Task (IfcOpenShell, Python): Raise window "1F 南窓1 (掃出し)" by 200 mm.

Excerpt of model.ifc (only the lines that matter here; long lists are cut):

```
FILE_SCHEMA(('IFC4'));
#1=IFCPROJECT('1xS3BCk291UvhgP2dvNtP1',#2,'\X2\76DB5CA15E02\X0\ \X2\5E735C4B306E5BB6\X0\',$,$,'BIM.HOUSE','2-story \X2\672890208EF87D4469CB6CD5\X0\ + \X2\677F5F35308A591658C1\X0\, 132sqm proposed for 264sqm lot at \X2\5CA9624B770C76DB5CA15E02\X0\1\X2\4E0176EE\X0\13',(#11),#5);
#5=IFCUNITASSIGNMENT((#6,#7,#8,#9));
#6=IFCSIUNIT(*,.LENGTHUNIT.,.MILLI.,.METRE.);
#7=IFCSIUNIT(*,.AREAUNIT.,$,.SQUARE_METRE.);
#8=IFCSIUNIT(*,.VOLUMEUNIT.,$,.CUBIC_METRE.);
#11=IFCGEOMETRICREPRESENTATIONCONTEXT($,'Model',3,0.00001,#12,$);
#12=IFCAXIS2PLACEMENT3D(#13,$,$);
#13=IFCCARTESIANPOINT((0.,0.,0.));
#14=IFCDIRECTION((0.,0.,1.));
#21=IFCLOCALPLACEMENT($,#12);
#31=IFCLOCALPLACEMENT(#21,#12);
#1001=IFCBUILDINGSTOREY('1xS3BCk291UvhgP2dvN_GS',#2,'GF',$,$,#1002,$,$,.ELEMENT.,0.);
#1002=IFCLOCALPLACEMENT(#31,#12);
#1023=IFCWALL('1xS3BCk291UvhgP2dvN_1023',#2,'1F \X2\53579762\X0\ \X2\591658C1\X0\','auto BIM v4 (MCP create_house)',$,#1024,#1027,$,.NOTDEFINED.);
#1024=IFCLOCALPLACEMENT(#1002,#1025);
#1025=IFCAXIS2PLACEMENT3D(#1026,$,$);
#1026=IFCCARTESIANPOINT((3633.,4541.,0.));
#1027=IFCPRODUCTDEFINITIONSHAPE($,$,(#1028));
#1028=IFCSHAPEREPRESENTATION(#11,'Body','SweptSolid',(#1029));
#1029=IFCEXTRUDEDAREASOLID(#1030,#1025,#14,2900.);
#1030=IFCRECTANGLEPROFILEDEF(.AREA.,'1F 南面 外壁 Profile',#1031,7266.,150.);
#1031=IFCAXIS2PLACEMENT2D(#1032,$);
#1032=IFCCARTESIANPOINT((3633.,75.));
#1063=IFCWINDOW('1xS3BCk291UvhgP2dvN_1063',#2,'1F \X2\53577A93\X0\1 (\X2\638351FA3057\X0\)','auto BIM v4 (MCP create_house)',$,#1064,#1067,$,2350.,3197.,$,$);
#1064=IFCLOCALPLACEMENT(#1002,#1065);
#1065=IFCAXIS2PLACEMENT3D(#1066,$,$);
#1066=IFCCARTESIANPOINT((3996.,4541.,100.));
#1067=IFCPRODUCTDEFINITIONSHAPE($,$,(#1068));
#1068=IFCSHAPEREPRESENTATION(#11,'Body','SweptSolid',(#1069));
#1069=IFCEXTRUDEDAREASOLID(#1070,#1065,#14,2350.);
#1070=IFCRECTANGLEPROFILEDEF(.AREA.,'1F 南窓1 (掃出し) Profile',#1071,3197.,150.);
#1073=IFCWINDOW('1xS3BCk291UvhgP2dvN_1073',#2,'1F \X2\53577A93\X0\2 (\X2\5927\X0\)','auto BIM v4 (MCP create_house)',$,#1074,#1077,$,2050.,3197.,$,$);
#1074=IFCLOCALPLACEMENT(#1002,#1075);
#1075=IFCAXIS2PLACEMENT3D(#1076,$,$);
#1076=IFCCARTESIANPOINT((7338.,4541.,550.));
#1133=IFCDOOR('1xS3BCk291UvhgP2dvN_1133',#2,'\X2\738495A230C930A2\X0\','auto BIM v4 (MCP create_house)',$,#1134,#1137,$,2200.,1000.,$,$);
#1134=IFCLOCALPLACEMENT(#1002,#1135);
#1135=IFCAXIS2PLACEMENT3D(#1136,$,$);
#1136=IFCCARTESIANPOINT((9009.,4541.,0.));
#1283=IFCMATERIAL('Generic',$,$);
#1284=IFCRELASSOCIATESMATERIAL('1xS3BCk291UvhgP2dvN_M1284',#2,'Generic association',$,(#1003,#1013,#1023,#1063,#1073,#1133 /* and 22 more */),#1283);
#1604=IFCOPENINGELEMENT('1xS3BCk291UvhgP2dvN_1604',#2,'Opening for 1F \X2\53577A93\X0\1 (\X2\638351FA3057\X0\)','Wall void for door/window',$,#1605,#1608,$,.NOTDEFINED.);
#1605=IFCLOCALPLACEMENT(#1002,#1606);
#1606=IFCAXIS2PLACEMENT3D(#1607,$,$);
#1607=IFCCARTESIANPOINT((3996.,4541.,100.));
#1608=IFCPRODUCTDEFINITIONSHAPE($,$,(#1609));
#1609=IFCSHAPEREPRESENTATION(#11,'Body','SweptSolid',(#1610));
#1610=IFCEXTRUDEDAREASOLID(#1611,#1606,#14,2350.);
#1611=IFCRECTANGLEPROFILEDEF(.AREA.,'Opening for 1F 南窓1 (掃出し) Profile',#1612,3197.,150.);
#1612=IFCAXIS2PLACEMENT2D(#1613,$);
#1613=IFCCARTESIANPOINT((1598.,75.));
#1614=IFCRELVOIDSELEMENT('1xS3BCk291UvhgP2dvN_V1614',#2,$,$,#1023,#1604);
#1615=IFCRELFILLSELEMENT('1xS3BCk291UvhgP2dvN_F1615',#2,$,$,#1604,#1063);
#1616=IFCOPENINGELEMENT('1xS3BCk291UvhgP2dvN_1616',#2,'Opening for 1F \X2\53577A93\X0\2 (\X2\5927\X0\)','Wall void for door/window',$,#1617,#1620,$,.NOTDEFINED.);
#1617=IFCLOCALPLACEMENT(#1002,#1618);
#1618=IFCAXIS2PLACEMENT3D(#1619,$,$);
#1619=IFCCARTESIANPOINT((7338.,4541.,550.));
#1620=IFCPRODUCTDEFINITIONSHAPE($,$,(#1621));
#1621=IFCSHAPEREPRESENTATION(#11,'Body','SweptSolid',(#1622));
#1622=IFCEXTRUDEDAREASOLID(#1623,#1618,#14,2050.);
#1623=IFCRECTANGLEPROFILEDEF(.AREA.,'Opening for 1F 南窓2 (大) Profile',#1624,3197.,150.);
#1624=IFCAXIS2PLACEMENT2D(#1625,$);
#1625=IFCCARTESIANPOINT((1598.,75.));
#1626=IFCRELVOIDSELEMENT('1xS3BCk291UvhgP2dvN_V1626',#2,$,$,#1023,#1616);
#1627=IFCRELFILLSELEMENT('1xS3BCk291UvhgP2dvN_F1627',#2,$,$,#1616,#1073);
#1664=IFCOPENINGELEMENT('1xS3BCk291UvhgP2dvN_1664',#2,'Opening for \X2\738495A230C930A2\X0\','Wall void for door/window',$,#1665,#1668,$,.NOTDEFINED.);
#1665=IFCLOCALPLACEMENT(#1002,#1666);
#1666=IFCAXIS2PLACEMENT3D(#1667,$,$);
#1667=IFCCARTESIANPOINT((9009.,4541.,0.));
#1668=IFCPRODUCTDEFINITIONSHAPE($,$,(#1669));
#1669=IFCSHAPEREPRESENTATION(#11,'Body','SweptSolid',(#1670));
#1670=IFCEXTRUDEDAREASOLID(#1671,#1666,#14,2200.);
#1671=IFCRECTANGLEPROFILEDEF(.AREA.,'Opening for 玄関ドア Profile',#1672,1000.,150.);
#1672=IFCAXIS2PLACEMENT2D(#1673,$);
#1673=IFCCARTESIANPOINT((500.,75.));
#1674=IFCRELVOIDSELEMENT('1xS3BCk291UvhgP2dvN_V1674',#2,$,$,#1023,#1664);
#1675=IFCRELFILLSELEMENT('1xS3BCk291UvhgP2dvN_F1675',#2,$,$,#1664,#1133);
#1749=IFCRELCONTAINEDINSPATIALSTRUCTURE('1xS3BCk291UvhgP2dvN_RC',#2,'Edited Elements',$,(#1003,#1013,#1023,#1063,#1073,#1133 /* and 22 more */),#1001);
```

```python
import numpy as np
import ifcopenshell
import ifcopenshell.api.geometry
import ifcopenshell.util.placement
import ifcopenshell.util.unit

model = ifcopenshell.open("model.ifc")
unit_scale = ifcopenshell.util.unit.calculate_unit_scale(model)

window = model.by_guid("1xS3BCk291UvhgP2dvN_1063")
opening = window.FillsVoids[0].RelatingOpeningElement
dz = 0.2 / unit_scale

shift = np.array([0.0, 0.0, dz])
# The window is not placed relative to its opening, so move both.
for product in (opening, window):
    matrix = ifcopenshell.util.placement.get_local_placement(product.ObjectPlacement)
    matrix[:3, 3] += shift
    ifcopenshell.api.geometry.edit_object_placement(model, product=product, matrix=matrix, is_si=False)

print(f"moved by {dz * unit_scale:+.3f} m")

model.write("model_rev.ifc")
```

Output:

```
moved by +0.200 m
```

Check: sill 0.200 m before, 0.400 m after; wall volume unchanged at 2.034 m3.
